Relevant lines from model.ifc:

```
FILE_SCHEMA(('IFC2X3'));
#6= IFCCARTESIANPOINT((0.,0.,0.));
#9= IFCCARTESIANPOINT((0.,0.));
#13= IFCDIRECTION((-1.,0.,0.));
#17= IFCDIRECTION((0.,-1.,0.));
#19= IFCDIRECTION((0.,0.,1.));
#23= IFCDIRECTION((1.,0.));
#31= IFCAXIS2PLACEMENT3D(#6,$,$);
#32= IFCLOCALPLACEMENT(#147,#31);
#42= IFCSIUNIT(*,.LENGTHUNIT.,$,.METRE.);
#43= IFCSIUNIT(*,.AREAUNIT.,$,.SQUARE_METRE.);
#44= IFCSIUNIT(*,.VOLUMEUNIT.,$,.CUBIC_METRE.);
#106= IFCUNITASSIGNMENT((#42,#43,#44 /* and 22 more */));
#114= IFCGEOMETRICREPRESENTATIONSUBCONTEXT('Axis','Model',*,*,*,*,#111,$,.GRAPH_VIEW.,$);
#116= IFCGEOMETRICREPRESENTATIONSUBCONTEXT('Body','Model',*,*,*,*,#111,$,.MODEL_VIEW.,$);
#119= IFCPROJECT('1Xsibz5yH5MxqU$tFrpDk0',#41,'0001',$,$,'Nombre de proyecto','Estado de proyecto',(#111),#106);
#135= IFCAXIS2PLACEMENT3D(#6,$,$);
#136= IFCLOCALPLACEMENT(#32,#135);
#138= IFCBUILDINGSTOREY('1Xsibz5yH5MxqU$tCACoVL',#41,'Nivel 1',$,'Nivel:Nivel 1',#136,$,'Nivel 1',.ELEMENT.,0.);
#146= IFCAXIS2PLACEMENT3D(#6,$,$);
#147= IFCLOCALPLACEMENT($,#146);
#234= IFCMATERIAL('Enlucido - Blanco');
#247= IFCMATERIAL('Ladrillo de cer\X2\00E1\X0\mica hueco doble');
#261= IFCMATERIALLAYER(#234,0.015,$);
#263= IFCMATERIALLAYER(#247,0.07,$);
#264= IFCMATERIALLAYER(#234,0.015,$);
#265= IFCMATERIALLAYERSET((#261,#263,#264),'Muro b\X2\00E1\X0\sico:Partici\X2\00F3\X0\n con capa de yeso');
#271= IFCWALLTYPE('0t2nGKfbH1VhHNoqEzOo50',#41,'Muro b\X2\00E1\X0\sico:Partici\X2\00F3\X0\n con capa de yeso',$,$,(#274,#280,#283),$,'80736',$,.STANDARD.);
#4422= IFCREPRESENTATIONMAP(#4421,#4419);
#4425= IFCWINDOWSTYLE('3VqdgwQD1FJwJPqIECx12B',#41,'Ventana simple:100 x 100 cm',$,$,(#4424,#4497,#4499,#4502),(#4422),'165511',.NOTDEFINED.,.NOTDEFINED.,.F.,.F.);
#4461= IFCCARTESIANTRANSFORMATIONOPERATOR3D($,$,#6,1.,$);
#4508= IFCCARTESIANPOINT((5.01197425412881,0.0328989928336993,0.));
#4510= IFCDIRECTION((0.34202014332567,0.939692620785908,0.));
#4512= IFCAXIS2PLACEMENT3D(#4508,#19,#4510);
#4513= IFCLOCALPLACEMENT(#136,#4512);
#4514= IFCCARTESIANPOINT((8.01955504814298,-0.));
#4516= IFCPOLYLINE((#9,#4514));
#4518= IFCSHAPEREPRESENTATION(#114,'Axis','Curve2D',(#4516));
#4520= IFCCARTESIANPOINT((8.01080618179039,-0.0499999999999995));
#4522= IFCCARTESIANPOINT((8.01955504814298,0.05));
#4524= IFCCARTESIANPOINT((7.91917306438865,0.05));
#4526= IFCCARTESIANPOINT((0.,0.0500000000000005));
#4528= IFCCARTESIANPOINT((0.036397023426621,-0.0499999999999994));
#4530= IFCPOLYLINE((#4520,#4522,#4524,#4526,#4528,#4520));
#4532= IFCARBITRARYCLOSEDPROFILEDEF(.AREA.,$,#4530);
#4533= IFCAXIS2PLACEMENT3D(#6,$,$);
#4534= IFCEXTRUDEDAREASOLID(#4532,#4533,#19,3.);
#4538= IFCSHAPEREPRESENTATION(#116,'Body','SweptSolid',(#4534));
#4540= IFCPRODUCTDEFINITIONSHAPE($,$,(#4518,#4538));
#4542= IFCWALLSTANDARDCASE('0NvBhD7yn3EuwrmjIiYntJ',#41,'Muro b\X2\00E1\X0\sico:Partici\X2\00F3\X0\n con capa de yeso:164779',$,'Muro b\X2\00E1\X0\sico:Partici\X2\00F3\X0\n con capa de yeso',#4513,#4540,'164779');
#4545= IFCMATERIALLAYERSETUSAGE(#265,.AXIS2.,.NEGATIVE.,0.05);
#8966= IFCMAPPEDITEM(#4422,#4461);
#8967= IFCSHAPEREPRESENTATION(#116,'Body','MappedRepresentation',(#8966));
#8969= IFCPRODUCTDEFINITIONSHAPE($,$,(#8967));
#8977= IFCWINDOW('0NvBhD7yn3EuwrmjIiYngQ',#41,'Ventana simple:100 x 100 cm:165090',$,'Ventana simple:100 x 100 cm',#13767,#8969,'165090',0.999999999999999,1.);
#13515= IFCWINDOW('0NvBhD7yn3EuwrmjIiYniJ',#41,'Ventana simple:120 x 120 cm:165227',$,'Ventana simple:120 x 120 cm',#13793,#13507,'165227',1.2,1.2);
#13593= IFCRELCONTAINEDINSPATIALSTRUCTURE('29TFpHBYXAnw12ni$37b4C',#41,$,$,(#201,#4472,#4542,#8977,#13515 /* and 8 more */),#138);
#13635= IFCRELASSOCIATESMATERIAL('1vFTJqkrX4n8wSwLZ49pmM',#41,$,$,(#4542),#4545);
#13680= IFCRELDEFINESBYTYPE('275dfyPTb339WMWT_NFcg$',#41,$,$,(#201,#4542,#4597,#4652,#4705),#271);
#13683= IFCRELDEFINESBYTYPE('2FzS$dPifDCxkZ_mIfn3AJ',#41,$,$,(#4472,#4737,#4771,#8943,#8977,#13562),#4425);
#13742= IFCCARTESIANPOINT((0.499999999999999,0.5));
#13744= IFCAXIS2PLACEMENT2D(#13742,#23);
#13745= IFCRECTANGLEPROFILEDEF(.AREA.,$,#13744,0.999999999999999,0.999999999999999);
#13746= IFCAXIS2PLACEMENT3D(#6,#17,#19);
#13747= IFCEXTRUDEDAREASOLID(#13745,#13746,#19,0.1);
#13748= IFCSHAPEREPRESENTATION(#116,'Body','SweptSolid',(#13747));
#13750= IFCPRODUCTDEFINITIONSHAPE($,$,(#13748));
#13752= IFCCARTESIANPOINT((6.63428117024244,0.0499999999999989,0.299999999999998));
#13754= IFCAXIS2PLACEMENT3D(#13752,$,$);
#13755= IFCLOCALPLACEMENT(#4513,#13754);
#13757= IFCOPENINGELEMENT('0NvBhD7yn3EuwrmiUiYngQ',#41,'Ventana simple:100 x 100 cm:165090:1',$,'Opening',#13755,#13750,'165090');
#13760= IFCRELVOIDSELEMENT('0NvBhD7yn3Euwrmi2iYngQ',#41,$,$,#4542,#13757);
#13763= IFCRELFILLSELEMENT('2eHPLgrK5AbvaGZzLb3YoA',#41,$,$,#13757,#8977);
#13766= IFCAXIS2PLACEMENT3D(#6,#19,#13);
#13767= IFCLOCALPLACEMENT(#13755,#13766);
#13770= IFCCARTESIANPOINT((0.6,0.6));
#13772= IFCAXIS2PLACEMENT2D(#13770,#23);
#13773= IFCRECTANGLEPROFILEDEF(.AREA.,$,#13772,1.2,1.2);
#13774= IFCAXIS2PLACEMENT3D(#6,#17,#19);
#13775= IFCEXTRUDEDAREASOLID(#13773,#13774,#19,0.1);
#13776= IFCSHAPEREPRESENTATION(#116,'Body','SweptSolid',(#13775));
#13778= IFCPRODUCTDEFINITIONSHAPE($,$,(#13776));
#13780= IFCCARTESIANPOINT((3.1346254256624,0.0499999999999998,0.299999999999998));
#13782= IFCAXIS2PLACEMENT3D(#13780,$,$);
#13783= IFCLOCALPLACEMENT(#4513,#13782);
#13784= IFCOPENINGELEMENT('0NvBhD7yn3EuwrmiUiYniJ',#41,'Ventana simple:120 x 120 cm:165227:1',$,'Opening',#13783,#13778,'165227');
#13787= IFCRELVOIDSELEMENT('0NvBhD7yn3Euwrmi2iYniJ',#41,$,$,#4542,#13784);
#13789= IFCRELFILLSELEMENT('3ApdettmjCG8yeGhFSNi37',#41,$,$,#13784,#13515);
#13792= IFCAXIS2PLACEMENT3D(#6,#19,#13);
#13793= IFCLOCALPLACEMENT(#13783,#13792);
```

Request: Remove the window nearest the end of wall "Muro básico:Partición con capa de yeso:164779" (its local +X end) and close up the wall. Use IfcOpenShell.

```python
import ifcopenshell
import ifcopenshell.api.feature
import ifcopenshell.api.root
import ifcopenshell.geom
import ifcopenshell.util.shape

model = ifcopenshell.open("model.ifc")
settings = ifcopenshell.geom.settings()


def volume(element):
    """Net volume in cubic metres, openings subtracted."""
    shape = ifcopenshell.geom.create_shape(settings, element)
    return ifcopenshell.util.shape.get_volume(shape.geometry)


window = model.by_guid("0NvBhD7yn3EuwrmjIiYngQ")
opening = window.FillsVoids[0].RelatingOpeningElement
wall = opening.VoidsElements[0].RelatingBuildingElement
before = volume(wall)

ifcopenshell.api.root.remove_product(model, product=window)
ifcopenshell.api.feature.remove_feature(model, feature=opening)

after = volume(wall)

print(f"wall volume {before:.3f} -> {after:.3f} m3")

model.write("model-out.ifc")
```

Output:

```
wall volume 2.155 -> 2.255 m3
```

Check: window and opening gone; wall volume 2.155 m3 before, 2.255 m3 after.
